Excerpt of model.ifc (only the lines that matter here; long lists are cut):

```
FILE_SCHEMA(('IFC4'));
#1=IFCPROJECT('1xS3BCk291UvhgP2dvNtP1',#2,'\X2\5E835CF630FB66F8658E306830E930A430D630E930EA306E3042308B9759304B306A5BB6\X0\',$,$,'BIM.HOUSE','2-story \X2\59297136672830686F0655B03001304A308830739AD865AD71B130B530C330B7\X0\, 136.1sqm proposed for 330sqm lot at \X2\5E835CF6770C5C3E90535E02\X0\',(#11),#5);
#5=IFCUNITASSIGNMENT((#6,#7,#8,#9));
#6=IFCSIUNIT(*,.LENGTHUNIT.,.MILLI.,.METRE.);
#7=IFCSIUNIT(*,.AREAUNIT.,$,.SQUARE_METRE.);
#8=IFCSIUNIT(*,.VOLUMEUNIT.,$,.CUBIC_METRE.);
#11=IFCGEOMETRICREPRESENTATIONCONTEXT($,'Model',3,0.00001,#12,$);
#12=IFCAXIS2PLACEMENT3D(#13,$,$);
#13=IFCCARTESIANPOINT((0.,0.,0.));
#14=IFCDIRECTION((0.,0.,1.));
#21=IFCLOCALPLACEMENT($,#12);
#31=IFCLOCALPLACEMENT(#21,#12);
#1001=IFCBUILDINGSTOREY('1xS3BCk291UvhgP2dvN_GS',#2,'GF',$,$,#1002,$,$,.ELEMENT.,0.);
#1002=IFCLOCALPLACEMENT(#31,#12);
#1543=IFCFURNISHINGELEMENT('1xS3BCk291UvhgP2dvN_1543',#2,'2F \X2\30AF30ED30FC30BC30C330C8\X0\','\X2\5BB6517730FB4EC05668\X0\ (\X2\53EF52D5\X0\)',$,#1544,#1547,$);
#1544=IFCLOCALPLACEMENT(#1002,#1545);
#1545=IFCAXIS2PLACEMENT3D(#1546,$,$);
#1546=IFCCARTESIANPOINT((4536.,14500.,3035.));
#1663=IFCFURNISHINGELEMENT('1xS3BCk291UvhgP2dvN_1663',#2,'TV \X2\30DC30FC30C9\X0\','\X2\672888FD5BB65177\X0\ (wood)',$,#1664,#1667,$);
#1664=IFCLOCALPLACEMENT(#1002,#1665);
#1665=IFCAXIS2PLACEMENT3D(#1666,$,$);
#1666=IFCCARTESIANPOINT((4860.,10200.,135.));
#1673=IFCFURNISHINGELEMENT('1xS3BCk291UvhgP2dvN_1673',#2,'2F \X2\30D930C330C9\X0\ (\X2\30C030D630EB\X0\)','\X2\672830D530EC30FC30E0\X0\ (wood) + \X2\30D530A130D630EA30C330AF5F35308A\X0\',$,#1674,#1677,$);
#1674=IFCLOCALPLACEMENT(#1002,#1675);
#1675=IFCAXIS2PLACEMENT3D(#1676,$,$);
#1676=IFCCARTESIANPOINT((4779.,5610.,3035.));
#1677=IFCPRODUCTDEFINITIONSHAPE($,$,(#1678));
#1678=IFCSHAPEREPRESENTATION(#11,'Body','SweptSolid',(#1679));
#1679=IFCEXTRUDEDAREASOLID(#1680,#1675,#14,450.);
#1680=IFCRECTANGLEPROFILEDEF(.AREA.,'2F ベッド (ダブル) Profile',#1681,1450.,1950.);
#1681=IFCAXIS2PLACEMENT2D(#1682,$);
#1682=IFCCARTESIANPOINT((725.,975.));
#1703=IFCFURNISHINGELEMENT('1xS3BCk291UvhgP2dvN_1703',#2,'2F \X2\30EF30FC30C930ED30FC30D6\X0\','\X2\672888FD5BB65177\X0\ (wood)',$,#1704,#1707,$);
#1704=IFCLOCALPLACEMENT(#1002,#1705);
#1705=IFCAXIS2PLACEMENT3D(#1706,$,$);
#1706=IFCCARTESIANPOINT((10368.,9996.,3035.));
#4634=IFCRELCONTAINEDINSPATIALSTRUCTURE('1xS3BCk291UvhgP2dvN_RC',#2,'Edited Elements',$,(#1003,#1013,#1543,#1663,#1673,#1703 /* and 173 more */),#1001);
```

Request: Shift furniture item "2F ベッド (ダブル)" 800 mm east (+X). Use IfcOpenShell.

```python
import ifcopenshell
import ifcopenshell.api.geometry
import ifcopenshell.util.placement
import ifcopenshell.util.unit

model = ifcopenshell.open("model.ifc")
unit_scale = ifcopenshell.util.unit.calculate_unit_scale(model)

item = model.by_guid("1xS3BCk291UvhgP2dvN_1673")
matrix = ifcopenshell.util.placement.get_local_placement(item.ObjectPlacement)
matrix[0, 3] += 0.8 / unit_scale
ifcopenshell.api.geometry.edit_object_placement(model, product=item, matrix=matrix, is_si=False)

print(ifcopenshell.util.placement.get_local_placement(item.ObjectPlacement).round(3) + 0.0)

model.write("model_rev.ifc")
```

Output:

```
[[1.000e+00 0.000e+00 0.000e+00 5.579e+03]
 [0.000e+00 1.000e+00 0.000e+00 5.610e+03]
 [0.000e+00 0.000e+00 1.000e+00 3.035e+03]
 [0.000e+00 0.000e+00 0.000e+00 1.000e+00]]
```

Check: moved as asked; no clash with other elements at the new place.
